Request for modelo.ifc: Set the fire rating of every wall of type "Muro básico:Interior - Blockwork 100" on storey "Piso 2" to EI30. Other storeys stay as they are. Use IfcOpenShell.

First a look at what the model holds.

```python
import ifcopenshell
import ifcopenshell.util.element

model = ifcopenshell.open("modelo.ifc")
print(model.schema)
storey = next(s for s in model.by_type("IfcBuildingStorey") if s.Name == "Piso 2")
walls = [e for e in ifcopenshell.util.element.get_decomposition(storey) if e.is_a("IfcWall")]
seen = {}
for e in walls:
    element_type = ifcopenshell.util.element.get_type(e)
    key = (element_type.Name if element_type != e and element_type else None, ifcopenshell.util.element.get_pset(e, "Pset_WallCommon", "FireRating"))
    seen[key] = seen.get(key, 0) + 1
for (name, value), count in sorted(seen.items(), key=str):
    print(count, "x", name, "|", value)
```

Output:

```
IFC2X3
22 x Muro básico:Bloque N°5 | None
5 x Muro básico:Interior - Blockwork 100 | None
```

```python
import ifcopenshell
import ifcopenshell.api.pset
import ifcopenshell.util.element

model = ifcopenshell.open("modelo.ifc")

storey = next(s for s in model.by_type("IfcBuildingStorey") if s.Name == "Piso 2")
walls = [e for e in ifcopenshell.util.element.get_decomposition(storey) if e.is_a("IfcWall")]

count = 0
for e in walls:
    element_type = ifcopenshell.util.element.get_type(e)
    if element_type in (None, e) or element_type.Name != "Muro básico:Interior - Blockwork 100":
        continue
    # add_pset returns the element's existing set when there is one.
    pset = ifcopenshell.api.pset.add_pset(model, product=e, name="Pset_WallCommon")
    ifcopenshell.api.pset.edit_pset(model, pset=pset, properties={"FireRating": "EI30"})
    count += 1

print(count, "walls updated")

model.write("modelo_rev.ifc")
```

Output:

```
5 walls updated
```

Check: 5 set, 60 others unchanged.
